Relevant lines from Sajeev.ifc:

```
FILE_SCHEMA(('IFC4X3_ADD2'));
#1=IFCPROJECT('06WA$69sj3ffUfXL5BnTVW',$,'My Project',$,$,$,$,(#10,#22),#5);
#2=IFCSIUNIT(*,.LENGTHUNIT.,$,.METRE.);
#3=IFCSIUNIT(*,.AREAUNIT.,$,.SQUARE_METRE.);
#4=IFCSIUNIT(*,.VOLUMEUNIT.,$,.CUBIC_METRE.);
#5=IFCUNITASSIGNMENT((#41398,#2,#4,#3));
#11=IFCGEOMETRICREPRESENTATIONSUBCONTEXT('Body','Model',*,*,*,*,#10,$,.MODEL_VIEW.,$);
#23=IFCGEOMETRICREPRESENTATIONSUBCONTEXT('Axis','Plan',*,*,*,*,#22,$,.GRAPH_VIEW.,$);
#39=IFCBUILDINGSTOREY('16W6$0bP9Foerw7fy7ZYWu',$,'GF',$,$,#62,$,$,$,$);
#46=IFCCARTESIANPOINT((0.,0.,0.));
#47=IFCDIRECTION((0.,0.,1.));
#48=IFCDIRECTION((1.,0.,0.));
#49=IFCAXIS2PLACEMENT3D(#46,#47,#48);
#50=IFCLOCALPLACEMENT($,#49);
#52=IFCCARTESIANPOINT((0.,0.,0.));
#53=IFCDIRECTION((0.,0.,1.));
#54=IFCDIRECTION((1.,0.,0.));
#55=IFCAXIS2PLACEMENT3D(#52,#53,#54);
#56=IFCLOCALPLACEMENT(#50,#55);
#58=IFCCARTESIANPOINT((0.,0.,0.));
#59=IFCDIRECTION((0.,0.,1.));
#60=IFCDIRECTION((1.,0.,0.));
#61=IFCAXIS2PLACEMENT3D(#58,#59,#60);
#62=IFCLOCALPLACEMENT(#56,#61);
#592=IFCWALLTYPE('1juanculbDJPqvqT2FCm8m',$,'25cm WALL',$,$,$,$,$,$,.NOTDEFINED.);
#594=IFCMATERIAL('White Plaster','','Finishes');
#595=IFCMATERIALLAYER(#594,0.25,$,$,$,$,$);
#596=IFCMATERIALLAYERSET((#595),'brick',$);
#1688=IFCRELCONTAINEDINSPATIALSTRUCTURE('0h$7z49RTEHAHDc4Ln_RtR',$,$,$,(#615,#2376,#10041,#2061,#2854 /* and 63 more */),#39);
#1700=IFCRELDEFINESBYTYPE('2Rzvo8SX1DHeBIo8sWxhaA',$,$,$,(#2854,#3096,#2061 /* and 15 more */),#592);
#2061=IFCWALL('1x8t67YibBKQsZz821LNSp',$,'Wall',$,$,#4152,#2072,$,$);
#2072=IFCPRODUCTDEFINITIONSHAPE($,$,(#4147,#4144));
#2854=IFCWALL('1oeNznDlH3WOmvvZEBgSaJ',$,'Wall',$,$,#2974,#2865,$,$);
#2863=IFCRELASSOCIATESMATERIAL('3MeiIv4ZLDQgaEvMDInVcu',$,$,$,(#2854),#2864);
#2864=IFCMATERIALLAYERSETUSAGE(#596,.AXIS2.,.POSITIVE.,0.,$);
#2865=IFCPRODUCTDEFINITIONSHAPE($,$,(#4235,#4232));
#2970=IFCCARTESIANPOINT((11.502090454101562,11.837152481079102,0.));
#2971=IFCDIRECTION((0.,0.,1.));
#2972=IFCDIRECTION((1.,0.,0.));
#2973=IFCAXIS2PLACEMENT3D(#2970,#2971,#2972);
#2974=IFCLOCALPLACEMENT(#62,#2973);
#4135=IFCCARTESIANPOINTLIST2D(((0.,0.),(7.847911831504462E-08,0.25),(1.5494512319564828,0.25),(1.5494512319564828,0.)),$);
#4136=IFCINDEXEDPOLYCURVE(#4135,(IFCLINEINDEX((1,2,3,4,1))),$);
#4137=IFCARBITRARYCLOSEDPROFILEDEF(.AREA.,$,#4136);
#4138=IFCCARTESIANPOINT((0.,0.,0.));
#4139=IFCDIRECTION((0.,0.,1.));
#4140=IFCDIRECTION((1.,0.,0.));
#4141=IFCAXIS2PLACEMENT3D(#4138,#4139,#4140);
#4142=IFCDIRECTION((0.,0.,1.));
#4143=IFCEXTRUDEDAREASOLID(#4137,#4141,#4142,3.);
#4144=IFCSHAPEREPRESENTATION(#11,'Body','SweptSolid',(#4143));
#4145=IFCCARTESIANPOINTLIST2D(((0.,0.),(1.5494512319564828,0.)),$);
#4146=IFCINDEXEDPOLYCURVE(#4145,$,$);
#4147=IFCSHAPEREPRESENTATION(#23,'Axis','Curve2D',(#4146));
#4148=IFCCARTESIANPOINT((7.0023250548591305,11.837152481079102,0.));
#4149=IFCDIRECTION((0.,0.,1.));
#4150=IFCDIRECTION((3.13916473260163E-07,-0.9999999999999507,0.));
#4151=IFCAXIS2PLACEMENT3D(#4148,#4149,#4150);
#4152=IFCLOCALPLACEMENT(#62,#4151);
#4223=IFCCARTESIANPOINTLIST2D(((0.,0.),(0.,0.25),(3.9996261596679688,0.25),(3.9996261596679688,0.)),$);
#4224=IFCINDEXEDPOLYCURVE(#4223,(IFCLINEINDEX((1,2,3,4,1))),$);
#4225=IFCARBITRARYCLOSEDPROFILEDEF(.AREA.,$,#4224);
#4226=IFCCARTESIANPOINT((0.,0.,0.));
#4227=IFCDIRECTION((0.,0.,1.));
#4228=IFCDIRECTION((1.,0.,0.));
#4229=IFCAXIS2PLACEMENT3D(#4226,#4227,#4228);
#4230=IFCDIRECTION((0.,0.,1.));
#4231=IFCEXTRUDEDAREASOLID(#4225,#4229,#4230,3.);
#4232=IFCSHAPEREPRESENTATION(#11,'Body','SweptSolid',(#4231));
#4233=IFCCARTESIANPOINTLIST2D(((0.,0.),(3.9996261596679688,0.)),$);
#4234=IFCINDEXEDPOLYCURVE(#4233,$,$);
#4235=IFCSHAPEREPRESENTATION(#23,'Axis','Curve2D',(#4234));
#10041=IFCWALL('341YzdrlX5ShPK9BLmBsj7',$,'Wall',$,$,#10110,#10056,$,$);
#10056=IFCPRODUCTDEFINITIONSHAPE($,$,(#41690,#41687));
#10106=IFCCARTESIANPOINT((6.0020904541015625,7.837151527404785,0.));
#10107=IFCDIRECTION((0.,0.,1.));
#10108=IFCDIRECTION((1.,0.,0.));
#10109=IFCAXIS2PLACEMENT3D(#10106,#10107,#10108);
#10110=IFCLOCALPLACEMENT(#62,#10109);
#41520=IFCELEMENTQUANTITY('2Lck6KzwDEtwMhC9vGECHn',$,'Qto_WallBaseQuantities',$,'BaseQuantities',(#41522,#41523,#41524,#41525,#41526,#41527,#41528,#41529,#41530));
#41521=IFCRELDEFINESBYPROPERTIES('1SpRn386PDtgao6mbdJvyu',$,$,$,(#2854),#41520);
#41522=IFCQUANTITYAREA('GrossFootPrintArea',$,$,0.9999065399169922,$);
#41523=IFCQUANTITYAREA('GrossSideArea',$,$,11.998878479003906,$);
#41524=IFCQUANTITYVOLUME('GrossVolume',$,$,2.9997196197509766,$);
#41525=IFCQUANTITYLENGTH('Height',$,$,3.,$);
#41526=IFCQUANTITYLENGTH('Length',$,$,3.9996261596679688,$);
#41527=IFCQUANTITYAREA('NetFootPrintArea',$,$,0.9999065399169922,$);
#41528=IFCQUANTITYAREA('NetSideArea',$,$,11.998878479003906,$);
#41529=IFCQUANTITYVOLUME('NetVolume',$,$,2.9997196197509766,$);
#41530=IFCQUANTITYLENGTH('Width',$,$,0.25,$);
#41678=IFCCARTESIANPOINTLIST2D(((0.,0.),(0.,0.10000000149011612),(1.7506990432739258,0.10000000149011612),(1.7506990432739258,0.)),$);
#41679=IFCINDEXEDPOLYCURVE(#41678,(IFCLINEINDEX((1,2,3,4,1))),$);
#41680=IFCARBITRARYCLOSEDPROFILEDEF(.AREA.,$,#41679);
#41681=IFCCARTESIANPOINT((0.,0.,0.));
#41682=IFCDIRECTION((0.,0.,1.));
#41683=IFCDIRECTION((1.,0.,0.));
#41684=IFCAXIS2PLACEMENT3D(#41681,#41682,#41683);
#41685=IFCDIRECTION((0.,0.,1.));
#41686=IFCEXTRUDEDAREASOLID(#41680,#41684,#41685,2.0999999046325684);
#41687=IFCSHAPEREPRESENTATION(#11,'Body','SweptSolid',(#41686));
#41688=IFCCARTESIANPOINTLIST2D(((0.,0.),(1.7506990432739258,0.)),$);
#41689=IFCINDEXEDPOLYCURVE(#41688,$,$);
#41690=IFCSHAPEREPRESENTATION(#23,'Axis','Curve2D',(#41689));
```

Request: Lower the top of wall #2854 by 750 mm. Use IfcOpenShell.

```python
import ifcopenshell
import ifcopenshell.api.pset
import ifcopenshell.geom
import ifcopenshell.util.element
import ifcopenshell.util.representation
import ifcopenshell.util.shape
import ifcopenshell.util.unit

model = ifcopenshell.open("Sajeev.ifc")
unit_scale = ifcopenshell.util.unit.calculate_unit_scale(model)
area_scale = ifcopenshell.util.unit.calculate_unit_scale(model, "AREAUNIT")
volume_scale = ifcopenshell.util.unit.calculate_unit_scale(model, "VOLUMEUNIT")
settings = ifcopenshell.geom.settings()


def volume(element):
    """Net volume in cubic metres, openings subtracted."""
    shape = ifcopenshell.geom.create_shape(settings, element)
    return ifcopenshell.util.shape.get_volume(shape.geometry)


wall = model.by_guid("1oeNznDlH3WOmvvZEBgSaJ")
before = volume(wall)

body = ifcopenshell.util.representation.get_representation(wall, "Model", "Body")
solid = body.Items[0]
old_height = solid.Depth
solid.Depth -= 0.75
after = volume(wall)
thickness = 0.25  # wall thickness in metres

# Update the stored height, areas and volumes.
qto = model.by_id(ifcopenshell.util.element.get_pset(wall, "Qto_WallBaseQuantities", should_inherit=False)["id"])
ifcopenshell.api.pset.edit_qto(model, qto=qto, properties={
    "GrossSideArea": ifcopenshell.util.element.get_pset(wall, "Qto_WallBaseQuantities", "GrossSideArea") * solid.Depth / old_height,
    "GrossVolume": ifcopenshell.util.element.get_pset(wall, "Qto_WallBaseQuantities", "GrossVolume") * solid.Depth / old_height,
    "Height": solid.Depth,
    "NetSideArea": after / thickness / area_scale,
    "NetVolume": after / volume_scale,
})

print(f"height {old_height:g} -> {solid.Depth:g}, volume {before:.3f} -> {after:.3f} m3")

model.write("Sajeev_v2.ifc")
```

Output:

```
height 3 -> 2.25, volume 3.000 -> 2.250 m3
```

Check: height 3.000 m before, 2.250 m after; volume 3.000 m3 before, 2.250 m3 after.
